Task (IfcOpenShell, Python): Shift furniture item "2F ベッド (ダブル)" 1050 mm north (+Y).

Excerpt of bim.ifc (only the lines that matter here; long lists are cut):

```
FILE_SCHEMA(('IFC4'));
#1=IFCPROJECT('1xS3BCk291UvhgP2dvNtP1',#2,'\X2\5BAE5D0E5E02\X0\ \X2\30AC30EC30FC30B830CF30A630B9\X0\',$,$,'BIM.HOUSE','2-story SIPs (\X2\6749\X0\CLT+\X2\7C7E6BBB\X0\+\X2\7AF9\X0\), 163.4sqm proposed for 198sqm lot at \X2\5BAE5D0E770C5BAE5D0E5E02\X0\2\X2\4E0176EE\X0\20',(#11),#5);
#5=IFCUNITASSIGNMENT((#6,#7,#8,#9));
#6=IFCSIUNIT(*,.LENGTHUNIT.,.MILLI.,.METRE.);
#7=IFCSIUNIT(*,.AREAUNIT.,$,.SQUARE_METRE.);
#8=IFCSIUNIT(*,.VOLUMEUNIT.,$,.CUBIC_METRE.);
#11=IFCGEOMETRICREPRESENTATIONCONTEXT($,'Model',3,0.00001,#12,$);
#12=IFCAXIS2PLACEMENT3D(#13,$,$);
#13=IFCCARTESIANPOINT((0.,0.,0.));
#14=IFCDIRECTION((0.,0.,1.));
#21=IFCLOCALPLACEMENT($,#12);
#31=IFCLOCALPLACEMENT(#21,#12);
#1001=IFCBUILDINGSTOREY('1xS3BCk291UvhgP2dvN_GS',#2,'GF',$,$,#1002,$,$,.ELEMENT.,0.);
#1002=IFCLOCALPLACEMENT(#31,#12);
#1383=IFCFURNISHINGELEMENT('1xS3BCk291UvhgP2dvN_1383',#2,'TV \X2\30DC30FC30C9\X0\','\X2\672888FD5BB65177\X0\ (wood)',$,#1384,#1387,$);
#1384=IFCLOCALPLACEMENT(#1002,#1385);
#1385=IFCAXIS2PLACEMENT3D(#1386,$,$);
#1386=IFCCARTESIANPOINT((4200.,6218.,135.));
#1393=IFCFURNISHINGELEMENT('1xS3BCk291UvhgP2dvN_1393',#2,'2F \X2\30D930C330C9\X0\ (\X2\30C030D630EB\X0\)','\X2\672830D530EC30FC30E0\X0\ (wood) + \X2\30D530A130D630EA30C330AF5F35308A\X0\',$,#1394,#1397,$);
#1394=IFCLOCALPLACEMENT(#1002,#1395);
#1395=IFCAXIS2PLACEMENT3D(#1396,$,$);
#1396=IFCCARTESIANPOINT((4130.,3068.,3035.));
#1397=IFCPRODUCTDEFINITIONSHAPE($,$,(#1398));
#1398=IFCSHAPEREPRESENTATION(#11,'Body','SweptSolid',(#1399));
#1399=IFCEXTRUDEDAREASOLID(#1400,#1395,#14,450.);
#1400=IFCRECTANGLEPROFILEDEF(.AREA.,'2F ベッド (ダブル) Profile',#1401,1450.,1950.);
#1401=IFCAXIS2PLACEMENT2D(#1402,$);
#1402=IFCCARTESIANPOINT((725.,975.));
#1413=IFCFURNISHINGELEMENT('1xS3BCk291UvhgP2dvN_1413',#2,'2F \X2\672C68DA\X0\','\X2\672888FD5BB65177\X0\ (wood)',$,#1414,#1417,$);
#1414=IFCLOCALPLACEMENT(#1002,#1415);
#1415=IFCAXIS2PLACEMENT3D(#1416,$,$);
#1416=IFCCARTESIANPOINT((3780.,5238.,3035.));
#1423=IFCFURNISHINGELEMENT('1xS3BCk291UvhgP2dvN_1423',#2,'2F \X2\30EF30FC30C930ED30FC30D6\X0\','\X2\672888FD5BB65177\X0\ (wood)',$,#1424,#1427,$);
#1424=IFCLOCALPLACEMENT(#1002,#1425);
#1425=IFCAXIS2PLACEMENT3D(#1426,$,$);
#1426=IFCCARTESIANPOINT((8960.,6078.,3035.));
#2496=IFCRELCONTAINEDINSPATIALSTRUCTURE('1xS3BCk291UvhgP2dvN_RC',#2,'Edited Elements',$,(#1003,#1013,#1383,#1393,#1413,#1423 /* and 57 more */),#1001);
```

```python
import ifcopenshell
import ifcopenshell.api.geometry
import ifcopenshell.util.placement

model = ifcopenshell.open("bim.ifc")

item = model.by_guid("1xS3BCk291UvhgP2dvN_1393")
matrix = ifcopenshell.util.placement.get_local_placement(item.ObjectPlacement)
matrix[1, 3] += 1050.0
ifcopenshell.api.geometry.edit_object_placement(model, product=item, matrix=matrix, is_si=False)

print(ifcopenshell.util.placement.get_local_placement(item.ObjectPlacement).round(3) + 0.0)

model.write("bim_edited.ifc")
```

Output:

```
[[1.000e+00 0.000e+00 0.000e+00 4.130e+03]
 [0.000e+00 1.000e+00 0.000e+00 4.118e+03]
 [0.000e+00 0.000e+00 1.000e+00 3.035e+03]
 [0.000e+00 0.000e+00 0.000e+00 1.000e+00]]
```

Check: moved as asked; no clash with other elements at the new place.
